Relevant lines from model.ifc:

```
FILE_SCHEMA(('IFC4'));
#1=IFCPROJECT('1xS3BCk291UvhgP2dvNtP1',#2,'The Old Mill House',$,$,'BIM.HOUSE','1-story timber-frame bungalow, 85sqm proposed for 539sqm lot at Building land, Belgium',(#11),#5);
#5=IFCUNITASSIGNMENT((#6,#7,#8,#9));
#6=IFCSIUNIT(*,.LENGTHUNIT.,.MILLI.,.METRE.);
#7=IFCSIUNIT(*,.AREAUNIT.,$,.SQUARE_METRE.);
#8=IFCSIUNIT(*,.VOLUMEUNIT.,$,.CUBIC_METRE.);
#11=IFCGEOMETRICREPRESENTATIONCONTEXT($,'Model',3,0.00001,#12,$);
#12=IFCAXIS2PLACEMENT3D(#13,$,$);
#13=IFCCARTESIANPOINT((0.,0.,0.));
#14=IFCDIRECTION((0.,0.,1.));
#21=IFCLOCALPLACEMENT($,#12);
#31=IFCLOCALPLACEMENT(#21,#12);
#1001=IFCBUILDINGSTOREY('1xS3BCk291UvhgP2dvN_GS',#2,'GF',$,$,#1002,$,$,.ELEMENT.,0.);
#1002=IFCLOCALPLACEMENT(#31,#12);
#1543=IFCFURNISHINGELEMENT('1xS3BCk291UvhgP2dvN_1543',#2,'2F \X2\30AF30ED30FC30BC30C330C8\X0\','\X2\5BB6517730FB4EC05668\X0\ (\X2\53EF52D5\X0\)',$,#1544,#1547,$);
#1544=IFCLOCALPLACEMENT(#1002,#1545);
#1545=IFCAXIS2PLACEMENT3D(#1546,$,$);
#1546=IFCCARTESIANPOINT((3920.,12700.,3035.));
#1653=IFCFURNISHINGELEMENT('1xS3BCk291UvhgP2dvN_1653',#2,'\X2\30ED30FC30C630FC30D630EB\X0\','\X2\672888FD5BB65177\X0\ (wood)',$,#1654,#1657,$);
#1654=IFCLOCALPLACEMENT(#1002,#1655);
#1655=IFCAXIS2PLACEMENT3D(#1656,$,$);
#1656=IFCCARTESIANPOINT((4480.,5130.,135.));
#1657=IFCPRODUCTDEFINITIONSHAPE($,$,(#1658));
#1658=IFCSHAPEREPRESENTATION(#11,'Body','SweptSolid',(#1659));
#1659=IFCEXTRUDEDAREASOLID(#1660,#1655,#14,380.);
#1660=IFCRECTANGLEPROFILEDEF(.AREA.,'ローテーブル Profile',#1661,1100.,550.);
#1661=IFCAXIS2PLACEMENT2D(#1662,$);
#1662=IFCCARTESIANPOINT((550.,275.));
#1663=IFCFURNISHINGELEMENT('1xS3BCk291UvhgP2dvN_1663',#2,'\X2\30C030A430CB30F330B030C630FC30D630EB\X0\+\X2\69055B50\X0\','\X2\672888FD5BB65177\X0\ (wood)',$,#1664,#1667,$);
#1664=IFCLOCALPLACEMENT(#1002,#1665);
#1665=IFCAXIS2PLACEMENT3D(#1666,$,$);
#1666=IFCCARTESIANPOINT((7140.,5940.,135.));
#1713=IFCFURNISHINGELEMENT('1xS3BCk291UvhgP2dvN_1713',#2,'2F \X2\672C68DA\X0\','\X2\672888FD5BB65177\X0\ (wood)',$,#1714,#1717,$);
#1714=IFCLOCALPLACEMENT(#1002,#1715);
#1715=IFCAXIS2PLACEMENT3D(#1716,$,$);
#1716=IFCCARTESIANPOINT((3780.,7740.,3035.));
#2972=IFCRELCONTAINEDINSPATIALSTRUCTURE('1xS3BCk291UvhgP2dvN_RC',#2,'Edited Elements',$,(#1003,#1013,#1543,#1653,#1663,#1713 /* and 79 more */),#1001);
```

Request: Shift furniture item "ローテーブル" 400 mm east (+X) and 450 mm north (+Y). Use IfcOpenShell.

```python
import ifcopenshell
import ifcopenshell.api.geometry
import ifcopenshell.util.placement

model = ifcopenshell.open("model.ifc")

item = model.by_guid("1xS3BCk291UvhgP2dvN_1653")
matrix = ifcopenshell.util.placement.get_local_placement(item.ObjectPlacement)
matrix[0, 3] += 400.0
matrix[1, 3] += 450.0
ifcopenshell.api.geometry.edit_object_placement(model, product=item, matrix=matrix, is_si=False)

print(ifcopenshell.util.placement.get_local_placement(item.ObjectPlacement).round(3) + 0.0)

model.write("model-out.ifc")
```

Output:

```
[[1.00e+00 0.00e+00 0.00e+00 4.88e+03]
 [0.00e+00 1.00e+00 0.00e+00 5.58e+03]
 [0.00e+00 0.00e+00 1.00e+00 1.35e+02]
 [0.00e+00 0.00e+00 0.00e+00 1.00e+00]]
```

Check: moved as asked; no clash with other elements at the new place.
